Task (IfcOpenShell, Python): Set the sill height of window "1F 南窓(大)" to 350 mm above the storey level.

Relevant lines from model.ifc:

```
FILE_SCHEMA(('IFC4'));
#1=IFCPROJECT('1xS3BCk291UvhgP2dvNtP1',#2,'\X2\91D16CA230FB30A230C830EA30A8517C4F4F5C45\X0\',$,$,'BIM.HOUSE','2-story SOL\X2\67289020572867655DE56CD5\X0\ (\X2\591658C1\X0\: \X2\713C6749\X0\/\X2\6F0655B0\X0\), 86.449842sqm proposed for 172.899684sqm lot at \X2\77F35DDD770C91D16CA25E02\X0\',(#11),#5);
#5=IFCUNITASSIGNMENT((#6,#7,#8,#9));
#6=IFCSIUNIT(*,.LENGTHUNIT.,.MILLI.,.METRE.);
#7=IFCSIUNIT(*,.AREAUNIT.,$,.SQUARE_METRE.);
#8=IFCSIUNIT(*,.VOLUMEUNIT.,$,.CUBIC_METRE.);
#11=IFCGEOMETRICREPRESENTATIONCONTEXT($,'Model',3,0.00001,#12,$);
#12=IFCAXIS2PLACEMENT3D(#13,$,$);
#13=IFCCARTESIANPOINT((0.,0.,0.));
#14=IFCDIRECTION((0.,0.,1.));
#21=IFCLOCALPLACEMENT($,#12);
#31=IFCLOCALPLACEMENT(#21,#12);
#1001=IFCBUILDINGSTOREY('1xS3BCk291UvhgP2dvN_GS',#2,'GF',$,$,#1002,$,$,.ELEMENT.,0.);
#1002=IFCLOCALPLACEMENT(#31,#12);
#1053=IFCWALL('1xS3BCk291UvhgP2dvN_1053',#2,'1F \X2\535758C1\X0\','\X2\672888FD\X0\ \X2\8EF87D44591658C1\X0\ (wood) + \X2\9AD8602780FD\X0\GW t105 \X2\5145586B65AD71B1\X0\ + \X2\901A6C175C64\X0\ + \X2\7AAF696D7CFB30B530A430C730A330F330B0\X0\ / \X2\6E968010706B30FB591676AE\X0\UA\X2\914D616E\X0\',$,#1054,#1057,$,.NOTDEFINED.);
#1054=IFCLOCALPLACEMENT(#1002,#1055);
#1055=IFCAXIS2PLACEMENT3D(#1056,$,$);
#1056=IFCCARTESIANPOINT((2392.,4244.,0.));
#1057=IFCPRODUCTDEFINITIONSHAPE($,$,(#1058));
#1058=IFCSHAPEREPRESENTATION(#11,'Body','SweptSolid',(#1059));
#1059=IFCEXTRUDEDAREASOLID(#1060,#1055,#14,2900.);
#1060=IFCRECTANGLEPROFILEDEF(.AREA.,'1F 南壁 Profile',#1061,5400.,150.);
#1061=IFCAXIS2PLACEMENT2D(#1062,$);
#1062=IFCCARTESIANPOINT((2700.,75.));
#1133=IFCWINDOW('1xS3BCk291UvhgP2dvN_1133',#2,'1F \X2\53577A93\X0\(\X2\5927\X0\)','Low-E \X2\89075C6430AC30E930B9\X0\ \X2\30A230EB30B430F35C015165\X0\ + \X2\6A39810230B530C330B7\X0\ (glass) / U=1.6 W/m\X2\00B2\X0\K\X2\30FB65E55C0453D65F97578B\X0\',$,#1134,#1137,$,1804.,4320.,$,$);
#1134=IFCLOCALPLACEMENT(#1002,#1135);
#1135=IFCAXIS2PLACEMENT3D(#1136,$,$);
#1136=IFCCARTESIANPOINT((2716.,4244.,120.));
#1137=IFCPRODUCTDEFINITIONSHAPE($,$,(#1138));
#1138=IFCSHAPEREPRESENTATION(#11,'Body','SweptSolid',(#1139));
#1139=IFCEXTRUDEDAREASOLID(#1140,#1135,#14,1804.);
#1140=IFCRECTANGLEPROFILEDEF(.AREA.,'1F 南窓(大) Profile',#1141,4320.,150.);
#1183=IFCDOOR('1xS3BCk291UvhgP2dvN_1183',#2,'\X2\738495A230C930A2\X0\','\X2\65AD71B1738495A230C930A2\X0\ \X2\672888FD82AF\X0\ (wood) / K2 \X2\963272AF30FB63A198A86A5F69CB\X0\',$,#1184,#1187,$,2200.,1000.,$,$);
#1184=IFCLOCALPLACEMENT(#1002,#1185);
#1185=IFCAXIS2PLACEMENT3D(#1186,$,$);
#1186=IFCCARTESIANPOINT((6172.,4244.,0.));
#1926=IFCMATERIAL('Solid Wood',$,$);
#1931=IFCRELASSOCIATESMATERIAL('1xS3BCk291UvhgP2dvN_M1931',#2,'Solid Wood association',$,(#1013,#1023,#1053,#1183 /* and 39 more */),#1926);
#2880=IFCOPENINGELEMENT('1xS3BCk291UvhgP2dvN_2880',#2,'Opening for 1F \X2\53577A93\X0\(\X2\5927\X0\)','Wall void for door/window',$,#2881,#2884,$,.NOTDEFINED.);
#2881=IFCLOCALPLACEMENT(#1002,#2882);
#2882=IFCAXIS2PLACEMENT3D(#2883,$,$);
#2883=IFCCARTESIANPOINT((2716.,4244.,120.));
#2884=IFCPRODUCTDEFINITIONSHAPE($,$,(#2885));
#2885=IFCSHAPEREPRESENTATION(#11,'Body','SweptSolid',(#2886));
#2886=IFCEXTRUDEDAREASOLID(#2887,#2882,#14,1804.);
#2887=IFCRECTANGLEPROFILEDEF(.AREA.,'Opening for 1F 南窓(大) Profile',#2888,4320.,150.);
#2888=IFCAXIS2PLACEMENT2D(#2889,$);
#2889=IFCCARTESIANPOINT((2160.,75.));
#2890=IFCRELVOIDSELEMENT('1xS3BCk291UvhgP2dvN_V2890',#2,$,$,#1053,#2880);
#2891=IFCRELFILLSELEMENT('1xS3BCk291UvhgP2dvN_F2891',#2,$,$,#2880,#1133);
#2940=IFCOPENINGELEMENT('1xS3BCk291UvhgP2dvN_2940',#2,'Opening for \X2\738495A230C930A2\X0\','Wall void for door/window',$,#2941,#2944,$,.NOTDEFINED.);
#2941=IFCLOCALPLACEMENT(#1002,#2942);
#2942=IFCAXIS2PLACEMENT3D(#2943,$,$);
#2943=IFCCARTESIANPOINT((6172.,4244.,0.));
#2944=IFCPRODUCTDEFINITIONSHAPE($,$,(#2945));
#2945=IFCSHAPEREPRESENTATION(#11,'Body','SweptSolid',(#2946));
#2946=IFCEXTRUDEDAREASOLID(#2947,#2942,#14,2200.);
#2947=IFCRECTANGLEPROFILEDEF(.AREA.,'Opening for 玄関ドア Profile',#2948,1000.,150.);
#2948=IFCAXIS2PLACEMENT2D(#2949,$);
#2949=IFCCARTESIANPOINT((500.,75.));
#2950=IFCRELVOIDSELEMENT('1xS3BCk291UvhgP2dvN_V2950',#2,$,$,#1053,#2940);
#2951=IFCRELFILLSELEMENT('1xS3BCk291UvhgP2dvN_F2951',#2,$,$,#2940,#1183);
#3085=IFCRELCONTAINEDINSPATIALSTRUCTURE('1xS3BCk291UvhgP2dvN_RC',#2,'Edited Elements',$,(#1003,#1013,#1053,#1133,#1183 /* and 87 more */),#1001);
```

```python
import numpy as np
import ifcopenshell
import ifcopenshell.api.geometry
import ifcopenshell.geom
import ifcopenshell.util.element
import ifcopenshell.util.placement
import ifcopenshell.util.shape
import ifcopenshell.util.unit

model = ifcopenshell.open("model.ifc")
unit_scale = ifcopenshell.util.unit.calculate_unit_scale(model)

window = model.by_guid("1xS3BCk291UvhgP2dvN_1133")
opening = window.FillsVoids[0].RelatingOpeningElement
storey = ifcopenshell.util.element.get_container(window, ifc_class="IfcBuildingStorey")
level = ifcopenshell.util.placement.get_local_placement(storey.ObjectPlacement)[2, 3]

# The opening's origin need not be at the sill, so measure its lowest point.
shape = ifcopenshell.geom.create_shape(ifcopenshell.geom.settings(), opening)
bottom = ifcopenshell.util.shape.get_shape_bottom_elevation(shape, shape.geometry) / unit_scale
dz = level + 0.35 / unit_scale - bottom

shift = np.array([0.0, 0.0, dz])
# The window is not placed relative to its opening, so move both.
for product in (opening, window):
    matrix = ifcopenshell.util.placement.get_local_placement(product.ObjectPlacement)
    matrix[:3, 3] += shift
    ifcopenshell.api.geometry.edit_object_placement(model, product=product, matrix=matrix, is_si=False)

print(f"moved by {dz * unit_scale:+.3f} m")

model.write("model_updated.ifc")
```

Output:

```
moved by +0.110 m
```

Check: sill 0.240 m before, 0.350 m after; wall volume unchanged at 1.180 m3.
